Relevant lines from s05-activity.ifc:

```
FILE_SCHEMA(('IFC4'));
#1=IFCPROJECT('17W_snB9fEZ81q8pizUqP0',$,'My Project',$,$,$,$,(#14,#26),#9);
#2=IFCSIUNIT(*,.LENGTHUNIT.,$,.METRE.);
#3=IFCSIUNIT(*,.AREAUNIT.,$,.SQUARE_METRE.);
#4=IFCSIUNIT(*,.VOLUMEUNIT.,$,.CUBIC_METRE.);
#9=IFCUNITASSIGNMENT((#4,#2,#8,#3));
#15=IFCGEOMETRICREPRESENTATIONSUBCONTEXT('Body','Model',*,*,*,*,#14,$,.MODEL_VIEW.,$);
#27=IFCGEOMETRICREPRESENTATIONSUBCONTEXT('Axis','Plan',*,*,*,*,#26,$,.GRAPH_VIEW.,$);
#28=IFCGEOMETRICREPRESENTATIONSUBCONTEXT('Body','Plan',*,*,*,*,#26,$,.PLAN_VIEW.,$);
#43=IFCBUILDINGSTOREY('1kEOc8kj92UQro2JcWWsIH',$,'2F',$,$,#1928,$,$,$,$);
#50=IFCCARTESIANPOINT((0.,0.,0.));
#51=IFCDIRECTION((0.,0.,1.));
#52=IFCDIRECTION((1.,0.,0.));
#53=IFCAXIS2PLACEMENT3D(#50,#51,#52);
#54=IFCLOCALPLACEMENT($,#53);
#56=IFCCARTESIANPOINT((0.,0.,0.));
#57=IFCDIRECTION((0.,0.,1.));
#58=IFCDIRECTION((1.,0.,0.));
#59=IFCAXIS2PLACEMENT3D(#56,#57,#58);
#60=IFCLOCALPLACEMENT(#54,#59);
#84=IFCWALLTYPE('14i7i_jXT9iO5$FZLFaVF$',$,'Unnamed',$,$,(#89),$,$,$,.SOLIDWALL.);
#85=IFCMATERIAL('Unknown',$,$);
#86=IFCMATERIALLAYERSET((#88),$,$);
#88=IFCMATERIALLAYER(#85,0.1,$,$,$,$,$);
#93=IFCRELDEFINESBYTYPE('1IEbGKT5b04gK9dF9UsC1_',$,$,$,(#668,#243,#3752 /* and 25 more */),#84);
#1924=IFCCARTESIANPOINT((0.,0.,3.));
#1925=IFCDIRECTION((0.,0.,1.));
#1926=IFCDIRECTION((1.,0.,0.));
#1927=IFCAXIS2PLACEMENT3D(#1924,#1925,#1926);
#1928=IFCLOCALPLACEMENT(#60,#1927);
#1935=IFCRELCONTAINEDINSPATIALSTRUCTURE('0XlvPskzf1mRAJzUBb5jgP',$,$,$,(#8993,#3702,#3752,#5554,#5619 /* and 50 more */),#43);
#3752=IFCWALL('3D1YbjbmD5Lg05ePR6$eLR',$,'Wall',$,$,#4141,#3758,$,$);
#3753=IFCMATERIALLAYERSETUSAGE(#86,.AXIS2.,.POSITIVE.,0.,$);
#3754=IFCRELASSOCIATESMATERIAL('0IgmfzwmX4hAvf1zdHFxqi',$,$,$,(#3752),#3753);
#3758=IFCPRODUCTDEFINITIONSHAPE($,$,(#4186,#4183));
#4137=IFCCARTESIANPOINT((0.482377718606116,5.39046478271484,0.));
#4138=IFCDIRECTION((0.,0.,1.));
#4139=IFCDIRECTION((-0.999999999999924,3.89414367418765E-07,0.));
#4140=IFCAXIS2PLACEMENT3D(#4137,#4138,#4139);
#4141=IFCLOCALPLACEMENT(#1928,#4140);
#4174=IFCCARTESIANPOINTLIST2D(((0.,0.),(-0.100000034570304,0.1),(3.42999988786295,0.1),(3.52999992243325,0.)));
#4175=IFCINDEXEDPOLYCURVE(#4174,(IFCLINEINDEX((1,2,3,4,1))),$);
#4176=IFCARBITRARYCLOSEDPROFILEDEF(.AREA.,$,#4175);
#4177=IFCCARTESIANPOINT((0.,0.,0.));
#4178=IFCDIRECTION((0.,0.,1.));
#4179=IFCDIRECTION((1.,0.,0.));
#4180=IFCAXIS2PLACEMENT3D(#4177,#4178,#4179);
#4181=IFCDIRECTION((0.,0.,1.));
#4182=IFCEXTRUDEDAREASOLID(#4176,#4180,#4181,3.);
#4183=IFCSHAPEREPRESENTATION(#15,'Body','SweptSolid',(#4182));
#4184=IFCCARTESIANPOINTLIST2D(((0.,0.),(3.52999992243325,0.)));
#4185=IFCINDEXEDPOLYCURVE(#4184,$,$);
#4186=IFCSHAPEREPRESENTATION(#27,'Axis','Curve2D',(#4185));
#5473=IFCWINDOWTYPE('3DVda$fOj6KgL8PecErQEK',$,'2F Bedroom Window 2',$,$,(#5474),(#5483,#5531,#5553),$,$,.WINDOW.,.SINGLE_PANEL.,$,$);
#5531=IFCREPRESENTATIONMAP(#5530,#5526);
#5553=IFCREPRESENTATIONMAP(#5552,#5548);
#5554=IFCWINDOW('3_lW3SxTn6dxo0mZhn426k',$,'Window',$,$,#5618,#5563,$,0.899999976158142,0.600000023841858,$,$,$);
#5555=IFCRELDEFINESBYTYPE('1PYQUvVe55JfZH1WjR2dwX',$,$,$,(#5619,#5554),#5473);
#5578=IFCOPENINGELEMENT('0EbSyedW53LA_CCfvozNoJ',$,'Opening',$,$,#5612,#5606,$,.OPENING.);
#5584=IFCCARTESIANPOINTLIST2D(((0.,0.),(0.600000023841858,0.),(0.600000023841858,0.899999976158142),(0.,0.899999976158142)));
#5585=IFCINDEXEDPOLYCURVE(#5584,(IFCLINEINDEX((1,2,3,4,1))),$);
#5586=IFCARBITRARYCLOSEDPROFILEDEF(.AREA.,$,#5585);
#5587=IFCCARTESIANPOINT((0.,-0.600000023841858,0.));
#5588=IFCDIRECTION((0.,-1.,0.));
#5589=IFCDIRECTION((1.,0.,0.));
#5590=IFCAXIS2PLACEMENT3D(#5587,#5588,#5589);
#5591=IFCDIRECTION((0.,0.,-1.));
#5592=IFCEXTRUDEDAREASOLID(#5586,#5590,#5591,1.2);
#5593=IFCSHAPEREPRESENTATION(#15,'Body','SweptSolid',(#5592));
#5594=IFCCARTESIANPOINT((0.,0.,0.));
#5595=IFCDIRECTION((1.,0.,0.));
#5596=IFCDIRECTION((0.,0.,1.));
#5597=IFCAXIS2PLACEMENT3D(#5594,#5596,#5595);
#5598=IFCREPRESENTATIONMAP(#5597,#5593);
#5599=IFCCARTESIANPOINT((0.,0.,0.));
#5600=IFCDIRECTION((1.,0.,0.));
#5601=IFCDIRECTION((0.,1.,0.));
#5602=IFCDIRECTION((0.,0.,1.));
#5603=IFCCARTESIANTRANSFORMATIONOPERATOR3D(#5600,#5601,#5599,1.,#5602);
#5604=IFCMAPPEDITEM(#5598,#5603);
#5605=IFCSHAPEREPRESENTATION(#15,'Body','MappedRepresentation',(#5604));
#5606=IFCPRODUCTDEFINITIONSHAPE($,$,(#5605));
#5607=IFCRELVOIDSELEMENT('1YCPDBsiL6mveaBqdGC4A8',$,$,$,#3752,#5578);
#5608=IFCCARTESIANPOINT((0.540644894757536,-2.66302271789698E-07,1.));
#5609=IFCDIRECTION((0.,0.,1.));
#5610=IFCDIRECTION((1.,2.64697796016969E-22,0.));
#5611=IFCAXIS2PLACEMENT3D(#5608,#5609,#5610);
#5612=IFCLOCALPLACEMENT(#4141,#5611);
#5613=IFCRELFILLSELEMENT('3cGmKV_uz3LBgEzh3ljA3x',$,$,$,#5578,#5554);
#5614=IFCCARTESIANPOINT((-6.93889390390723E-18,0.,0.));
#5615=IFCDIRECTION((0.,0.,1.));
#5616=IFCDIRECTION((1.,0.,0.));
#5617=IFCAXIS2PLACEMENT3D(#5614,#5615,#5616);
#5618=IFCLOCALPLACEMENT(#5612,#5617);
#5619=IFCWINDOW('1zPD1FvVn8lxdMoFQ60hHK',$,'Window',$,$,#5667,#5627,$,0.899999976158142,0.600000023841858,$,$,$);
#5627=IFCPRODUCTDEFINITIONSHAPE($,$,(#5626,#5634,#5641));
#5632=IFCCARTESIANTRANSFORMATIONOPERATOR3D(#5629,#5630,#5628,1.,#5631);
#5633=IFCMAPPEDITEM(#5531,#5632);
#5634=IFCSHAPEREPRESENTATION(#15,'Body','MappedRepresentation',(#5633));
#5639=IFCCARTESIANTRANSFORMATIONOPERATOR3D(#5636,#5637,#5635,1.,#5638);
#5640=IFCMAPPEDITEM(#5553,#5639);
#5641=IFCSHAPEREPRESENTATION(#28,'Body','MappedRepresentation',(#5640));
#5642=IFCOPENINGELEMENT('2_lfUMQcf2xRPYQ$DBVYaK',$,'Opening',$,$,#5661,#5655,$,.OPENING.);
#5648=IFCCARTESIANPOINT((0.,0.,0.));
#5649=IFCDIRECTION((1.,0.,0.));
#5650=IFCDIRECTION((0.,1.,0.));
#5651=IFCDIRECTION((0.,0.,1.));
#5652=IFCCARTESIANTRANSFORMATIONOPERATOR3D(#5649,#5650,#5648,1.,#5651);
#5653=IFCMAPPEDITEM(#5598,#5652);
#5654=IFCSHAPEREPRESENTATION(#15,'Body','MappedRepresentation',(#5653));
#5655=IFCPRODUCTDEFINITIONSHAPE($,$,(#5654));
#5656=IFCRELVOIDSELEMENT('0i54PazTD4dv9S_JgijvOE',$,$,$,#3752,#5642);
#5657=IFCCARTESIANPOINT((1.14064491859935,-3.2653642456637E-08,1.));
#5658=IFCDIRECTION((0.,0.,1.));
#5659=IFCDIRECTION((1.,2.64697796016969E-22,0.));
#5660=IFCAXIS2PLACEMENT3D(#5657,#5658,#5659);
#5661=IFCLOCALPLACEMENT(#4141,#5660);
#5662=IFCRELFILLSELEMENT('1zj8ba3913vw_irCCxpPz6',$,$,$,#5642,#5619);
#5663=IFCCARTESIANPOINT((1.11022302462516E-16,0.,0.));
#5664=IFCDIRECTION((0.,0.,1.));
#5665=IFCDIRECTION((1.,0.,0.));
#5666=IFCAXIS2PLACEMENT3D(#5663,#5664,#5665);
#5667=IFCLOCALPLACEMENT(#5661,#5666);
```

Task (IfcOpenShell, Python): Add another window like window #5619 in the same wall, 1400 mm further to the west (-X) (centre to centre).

```python
import ifcopenshell
import ifcopenshell.api.feature
import ifcopenshell.api.geometry
import ifcopenshell.api.root
import ifcopenshell.geom
import ifcopenshell.util.element
import ifcopenshell.util.placement
import ifcopenshell.util.shape

model = ifcopenshell.open("s05-activity.ifc")
settings = ifcopenshell.geom.settings()


def volume(element):
    """Net volume in cubic metres, openings subtracted."""
    shape = ifcopenshell.geom.create_shape(settings, element)
    return ifcopenshell.util.shape.get_volume(shape.geometry)


window = model.by_id(5619)
opening = window.FillsVoids[0].RelatingOpeningElement
wall = opening.VoidsElements[0].RelatingBuildingElement
before = volume(wall)
shift = ifcopenshell.util.placement.get_local_placement(wall.ObjectPlacement)[:3, 0] * 1.4

# copy_class copies the void relationship, type, container and properties, but no geometry.
new_opening = ifcopenshell.api.root.copy_class(model, product=opening)
new_opening.Representation = ifcopenshell.util.element.copy_deep(
    model, opening.Representation, exclude=["IfcGeometricRepresentationContext", "IfcRepresentationMap"]
)
new_window = ifcopenshell.api.root.copy_class(model, product=window)
new_window.Representation = ifcopenshell.util.element.copy_deep(
    model, window.Representation, exclude=["IfcGeometricRepresentationContext", "IfcRepresentationMap"]
)
ifcopenshell.api.feature.add_filling(model, opening=new_opening, element=new_window)

for old, new in ((opening, new_opening), (window, new_window)):
    matrix = ifcopenshell.util.placement.get_local_placement(old.ObjectPlacement)
    matrix[:3, 3] += shift
    ifcopenshell.api.geometry.edit_object_placement(model, product=new, matrix=matrix, is_si=False)

after = volume(wall)

print(f"wall volume {before:.3f} -> {after:.3f} m3")

model.write("s05-activity_v2.ifc")
```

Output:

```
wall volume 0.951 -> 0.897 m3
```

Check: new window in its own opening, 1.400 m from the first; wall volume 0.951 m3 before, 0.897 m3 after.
